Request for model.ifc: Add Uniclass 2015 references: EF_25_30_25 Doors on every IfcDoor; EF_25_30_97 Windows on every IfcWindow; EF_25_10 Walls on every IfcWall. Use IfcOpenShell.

First a look at what the model holds.

```python
import ifcopenshell

model = ifcopenshell.open("model.ifc")
print(model.schema)
print("classifications:", [c.Name for c in model.by_type("IfcClassification")])
for ifc_class in ("IfcDoor", "IfcRoof", "IfcStair", "IfcWall", "IfcWindow"):
    print(ifc_class, len(model.by_type(ifc_class)))
```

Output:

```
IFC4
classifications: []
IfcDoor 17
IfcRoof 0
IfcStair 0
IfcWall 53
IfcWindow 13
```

```python
import ifcopenshell
import ifcopenshell.api.classification

model = ifcopenshell.open("model.ifc")

system = ifcopenshell.api.classification.add_classification(model, classification="Uniclass 2015")

codes = {
    "IfcDoor": ("EF_25_30_25", "Doors"),
    "IfcWindow": ("EF_25_30_97", "Windows"),
    "IfcWall": ("EF_25_10", "Walls"),
}
for ifc_class, (code, name) in codes.items():
    products = model.by_type(ifc_class)
    ifcopenshell.api.classification.add_reference(
        model, products=products, classification=system, identification=code, name=name
    )
    print(code, len(products))

model.write("model_rev.ifc")
```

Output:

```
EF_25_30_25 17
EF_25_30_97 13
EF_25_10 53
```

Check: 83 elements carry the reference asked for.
